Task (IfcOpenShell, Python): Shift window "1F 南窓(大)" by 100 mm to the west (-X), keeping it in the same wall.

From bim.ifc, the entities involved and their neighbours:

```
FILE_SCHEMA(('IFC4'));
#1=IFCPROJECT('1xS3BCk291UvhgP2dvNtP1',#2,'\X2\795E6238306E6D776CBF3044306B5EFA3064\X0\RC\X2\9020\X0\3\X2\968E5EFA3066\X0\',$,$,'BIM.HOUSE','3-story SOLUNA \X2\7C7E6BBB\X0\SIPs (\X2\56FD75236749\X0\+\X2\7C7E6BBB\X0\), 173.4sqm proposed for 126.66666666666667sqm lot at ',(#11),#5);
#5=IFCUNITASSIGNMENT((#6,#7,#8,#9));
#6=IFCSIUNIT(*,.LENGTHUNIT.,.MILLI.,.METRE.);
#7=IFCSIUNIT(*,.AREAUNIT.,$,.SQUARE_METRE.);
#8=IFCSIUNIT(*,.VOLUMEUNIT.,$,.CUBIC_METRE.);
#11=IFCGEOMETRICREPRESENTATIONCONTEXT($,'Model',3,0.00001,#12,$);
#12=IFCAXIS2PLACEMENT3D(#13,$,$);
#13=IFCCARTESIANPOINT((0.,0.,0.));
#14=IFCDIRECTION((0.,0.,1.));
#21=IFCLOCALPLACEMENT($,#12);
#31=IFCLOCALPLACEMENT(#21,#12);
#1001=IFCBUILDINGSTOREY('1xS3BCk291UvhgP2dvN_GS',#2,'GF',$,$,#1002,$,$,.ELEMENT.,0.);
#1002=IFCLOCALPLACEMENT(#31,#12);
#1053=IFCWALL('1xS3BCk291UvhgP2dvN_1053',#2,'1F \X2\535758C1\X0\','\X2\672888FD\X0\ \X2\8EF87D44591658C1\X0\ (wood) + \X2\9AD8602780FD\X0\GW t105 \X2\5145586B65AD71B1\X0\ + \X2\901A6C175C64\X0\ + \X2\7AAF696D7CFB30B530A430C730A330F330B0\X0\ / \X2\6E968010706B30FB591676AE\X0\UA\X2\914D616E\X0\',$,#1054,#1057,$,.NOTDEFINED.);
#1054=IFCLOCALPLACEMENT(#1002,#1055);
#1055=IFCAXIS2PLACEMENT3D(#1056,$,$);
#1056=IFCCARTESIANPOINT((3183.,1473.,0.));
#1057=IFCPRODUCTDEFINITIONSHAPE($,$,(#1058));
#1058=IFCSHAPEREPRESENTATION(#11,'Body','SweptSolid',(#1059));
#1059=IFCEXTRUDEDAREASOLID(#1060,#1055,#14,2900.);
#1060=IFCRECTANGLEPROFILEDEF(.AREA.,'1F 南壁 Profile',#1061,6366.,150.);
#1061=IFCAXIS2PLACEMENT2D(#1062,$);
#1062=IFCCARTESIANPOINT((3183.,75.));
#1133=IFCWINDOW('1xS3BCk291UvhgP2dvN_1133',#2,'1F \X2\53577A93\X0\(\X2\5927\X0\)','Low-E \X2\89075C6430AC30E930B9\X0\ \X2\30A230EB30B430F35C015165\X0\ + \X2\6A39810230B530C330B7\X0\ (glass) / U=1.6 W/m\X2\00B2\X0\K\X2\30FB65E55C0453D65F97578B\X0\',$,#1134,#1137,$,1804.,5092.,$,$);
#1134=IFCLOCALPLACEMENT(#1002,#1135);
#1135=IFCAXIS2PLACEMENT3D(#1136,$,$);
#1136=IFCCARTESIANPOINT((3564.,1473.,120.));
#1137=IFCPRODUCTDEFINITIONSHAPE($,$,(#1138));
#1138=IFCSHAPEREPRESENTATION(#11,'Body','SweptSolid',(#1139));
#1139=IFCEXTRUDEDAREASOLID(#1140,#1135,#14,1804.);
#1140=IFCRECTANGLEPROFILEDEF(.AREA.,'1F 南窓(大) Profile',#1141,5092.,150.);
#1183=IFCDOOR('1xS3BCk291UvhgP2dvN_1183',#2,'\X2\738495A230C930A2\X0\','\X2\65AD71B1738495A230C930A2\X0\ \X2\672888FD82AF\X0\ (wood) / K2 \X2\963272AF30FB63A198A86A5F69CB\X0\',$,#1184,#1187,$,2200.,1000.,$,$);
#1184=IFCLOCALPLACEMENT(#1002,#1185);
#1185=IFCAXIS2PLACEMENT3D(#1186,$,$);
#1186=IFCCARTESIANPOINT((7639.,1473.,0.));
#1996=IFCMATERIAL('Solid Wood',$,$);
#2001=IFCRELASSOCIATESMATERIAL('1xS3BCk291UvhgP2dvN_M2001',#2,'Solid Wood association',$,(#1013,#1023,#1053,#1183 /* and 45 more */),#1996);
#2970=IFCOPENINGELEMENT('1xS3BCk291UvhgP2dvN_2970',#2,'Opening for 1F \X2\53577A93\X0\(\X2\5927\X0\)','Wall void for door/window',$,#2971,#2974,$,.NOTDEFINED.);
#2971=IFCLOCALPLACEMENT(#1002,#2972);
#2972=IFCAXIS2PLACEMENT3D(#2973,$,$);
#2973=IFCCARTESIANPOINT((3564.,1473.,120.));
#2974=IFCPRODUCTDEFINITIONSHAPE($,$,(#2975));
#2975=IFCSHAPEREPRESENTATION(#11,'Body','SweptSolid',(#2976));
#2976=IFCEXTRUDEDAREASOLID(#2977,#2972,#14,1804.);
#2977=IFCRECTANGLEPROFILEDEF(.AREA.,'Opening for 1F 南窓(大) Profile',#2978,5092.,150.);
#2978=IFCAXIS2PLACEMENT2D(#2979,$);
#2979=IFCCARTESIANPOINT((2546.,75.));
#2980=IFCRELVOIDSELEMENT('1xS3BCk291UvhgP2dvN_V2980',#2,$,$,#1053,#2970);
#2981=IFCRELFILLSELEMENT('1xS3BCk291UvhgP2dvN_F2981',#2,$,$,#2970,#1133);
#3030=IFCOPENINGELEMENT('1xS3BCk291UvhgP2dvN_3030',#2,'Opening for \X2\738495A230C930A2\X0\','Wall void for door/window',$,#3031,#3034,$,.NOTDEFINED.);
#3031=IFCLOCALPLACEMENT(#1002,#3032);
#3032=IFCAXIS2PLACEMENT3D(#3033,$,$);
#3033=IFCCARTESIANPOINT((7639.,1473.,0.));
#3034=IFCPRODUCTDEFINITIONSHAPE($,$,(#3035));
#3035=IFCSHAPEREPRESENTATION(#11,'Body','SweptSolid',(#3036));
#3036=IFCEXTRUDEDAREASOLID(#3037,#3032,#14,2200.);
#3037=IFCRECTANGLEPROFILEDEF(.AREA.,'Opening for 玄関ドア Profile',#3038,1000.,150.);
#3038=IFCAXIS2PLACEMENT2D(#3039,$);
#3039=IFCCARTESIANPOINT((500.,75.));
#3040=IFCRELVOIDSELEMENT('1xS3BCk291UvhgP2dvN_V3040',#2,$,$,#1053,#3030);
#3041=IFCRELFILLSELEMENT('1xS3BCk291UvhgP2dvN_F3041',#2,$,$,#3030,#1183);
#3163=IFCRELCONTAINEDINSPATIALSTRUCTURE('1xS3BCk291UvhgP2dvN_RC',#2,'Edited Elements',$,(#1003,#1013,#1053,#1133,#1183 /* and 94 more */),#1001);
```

```python
import ifcopenshell
import ifcopenshell.api.geometry
import ifcopenshell.util.placement

model = ifcopenshell.open("bim.ifc")

window = model.by_guid("1xS3BCk291UvhgP2dvN_1133")
opening = window.FillsVoids[0].RelatingOpeningElement
wall = opening.VoidsElements[0].RelatingBuildingElement

wall_matrix = ifcopenshell.util.placement.get_local_placement(wall.ObjectPlacement)
shift = wall_matrix[:3, 0] * -100.0
before = ifcopenshell.util.placement.get_local_placement(window.ObjectPlacement)[:3, 3].copy()

# The window is not placed relative to its opening, so move both.
for product in (opening, window):
    matrix = ifcopenshell.util.placement.get_local_placement(product.ObjectPlacement)
    matrix[:3, 3] += shift
    ifcopenshell.api.geometry.edit_object_placement(model, product=product, matrix=matrix, is_si=False)

after = ifcopenshell.util.placement.get_local_placement(window.ObjectPlacement)[:3, 3]
print("window moved by", (after - before).round(3) + 0.0)

model.write("bim_rev.ifc")
```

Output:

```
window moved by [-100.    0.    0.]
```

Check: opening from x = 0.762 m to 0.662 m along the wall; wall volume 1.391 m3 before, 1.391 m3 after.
